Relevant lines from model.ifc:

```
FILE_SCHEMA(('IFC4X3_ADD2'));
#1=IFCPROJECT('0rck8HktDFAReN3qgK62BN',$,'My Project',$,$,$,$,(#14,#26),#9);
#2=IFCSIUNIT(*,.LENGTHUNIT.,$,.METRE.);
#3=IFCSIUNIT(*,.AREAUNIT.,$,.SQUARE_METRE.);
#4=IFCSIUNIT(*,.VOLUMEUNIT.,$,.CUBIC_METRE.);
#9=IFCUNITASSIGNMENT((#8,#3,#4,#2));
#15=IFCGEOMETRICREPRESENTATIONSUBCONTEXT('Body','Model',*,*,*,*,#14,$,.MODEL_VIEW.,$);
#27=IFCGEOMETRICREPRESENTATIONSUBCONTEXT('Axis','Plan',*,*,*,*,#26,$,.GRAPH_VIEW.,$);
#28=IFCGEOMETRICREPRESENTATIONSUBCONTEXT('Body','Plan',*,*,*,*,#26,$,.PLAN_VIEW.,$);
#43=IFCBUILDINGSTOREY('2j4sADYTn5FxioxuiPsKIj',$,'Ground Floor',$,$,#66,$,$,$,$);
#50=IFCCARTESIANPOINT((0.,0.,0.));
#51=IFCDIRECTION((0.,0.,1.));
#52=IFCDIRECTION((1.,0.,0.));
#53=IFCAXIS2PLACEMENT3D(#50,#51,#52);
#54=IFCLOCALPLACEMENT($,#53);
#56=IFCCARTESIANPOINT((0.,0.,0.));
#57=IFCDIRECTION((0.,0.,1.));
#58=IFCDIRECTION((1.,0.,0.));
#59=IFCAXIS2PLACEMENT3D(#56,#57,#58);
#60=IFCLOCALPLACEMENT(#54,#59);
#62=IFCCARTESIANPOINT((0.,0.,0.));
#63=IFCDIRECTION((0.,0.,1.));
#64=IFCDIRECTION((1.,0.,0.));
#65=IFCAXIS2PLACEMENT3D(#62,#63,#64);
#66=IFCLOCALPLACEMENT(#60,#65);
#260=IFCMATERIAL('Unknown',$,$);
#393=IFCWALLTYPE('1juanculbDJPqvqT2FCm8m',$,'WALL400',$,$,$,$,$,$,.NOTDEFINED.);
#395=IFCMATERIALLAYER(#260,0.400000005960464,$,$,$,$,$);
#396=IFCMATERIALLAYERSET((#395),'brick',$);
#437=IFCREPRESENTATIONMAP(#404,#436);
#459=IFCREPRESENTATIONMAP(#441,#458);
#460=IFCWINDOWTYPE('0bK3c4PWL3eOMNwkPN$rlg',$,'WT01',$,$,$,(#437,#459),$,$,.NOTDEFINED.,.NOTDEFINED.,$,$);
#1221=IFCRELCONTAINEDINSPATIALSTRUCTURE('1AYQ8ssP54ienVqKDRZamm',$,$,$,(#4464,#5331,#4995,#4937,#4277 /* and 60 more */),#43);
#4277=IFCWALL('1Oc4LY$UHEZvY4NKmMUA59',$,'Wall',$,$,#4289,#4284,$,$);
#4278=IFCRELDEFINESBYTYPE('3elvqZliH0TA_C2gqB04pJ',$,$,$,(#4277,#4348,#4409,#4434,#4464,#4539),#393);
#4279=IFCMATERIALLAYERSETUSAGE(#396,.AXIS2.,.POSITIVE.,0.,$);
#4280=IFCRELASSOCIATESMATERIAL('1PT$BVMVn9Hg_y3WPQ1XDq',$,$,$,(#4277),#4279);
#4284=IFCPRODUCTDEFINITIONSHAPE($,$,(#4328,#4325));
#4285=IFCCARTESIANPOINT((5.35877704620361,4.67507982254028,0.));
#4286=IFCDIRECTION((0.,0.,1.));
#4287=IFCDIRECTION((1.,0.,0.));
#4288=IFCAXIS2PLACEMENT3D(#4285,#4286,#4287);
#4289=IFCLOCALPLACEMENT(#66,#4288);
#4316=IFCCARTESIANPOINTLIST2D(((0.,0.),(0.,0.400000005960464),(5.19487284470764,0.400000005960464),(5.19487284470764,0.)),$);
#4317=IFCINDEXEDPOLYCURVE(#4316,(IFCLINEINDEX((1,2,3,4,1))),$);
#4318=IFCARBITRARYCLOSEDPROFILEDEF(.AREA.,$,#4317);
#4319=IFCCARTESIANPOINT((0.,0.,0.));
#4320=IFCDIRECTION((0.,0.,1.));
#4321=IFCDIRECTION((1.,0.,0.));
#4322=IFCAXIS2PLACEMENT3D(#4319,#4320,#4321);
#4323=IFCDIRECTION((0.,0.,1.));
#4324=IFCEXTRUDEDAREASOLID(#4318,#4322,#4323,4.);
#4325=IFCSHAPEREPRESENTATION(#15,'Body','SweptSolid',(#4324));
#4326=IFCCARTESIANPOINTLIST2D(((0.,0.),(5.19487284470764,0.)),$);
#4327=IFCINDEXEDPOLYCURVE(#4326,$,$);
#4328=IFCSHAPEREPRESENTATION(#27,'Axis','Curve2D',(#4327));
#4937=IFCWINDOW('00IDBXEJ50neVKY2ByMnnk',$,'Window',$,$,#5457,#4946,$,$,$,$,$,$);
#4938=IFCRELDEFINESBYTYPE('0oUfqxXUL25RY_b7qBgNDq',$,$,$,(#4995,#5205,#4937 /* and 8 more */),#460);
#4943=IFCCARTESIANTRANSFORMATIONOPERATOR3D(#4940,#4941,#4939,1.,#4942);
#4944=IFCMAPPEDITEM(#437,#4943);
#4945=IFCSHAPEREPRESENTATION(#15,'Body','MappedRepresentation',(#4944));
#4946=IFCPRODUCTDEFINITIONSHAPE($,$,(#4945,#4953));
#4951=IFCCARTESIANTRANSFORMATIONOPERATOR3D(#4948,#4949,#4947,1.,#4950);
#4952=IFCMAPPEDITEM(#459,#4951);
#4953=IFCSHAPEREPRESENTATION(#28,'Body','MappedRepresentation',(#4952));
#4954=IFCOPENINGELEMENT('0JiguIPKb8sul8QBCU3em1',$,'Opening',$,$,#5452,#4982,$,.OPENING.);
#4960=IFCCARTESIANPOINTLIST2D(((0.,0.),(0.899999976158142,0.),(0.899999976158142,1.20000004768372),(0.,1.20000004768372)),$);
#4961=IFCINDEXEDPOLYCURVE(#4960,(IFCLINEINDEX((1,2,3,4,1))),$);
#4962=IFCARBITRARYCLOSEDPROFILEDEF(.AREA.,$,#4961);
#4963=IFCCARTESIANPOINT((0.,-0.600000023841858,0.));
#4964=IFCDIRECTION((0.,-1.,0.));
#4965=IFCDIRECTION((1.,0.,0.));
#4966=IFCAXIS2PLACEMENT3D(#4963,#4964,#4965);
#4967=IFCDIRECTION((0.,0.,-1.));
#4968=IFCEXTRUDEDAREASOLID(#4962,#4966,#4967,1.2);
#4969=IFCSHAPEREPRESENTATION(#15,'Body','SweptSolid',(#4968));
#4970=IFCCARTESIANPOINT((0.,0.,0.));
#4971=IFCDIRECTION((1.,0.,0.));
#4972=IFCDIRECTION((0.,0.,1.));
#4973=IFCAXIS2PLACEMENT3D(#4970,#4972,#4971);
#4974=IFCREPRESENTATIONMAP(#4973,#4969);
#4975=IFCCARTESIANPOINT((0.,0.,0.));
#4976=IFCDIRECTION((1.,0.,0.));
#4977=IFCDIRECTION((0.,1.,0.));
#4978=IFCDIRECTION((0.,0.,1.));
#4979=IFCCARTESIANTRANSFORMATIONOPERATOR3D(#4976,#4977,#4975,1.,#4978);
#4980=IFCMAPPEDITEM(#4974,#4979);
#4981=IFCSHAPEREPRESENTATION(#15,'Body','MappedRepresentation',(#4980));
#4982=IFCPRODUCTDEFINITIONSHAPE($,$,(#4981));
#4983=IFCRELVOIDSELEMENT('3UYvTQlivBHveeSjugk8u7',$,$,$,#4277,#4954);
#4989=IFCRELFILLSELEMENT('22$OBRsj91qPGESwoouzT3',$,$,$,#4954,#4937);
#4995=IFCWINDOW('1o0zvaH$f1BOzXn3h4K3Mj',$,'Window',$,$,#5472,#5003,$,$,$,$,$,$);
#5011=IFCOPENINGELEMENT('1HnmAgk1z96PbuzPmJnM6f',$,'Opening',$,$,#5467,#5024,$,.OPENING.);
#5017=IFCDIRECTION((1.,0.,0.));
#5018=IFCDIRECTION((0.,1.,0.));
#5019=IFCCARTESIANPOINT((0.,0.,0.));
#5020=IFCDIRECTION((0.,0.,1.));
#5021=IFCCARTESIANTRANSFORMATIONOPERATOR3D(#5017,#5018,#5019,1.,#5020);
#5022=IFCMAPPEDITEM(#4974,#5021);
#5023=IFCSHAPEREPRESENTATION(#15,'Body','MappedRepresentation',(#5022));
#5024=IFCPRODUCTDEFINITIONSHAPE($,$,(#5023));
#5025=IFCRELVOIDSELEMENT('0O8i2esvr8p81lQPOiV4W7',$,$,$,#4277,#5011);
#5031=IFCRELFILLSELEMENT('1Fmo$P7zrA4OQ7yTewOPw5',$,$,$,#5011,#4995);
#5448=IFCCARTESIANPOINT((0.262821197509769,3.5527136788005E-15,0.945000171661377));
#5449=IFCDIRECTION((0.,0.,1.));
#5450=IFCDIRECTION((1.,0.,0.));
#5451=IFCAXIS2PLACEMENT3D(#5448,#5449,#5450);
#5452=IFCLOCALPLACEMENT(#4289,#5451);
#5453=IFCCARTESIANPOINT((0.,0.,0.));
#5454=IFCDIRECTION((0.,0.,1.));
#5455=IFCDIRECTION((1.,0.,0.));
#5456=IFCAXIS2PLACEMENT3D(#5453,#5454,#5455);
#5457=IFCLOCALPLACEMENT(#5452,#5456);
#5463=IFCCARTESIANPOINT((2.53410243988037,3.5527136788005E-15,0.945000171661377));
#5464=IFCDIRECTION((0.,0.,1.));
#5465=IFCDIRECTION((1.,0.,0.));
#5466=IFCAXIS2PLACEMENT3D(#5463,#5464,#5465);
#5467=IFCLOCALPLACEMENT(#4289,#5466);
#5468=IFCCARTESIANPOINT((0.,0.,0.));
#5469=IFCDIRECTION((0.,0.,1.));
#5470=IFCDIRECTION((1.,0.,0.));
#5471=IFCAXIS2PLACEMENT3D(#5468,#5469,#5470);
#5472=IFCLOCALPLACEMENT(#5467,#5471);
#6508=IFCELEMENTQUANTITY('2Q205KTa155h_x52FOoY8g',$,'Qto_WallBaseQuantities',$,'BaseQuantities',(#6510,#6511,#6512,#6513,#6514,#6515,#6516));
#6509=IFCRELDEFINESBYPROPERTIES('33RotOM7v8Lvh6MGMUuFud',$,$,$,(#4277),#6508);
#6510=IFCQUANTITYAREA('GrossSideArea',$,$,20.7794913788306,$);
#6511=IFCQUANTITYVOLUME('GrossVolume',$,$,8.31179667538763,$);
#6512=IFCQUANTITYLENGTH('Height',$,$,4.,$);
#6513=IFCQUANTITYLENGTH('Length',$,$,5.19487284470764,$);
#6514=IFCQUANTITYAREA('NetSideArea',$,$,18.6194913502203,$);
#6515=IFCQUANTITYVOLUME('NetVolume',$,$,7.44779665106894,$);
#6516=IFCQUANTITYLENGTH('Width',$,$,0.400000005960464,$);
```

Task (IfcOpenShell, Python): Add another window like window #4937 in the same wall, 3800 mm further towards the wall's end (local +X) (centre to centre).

```python
import ifcopenshell
import ifcopenshell.api.feature
import ifcopenshell.api.geometry
import ifcopenshell.api.pset
import ifcopenshell.api.root
import ifcopenshell.geom
import ifcopenshell.util.element
import ifcopenshell.util.placement
import ifcopenshell.util.shape
import ifcopenshell.util.unit

model = ifcopenshell.open("model.ifc")
unit_scale = ifcopenshell.util.unit.calculate_unit_scale(model)
area_scale = ifcopenshell.util.unit.calculate_unit_scale(model, "AREAUNIT")
volume_scale = ifcopenshell.util.unit.calculate_unit_scale(model, "VOLUMEUNIT")
settings = ifcopenshell.geom.settings()


def volume(element):
    """Net volume in cubic metres, openings subtracted."""
    shape = ifcopenshell.geom.create_shape(settings, element)
    return ifcopenshell.util.shape.get_volume(shape.geometry)


window = model.by_guid("00IDBXEJ50neVKY2ByMnnk")
opening = window.FillsVoids[0].RelatingOpeningElement
wall = opening.VoidsElements[0].RelatingBuildingElement
before = volume(wall)
shift = ifcopenshell.util.placement.get_local_placement(wall.ObjectPlacement)[:3, 0] * 3.8 / unit_scale

# copy_class copies the void relationship, type, container and properties, but no geometry.
new_opening = ifcopenshell.api.root.copy_class(model, product=opening)
new_opening.Representation = ifcopenshell.util.element.copy_deep(
    model, opening.Representation, exclude=["IfcGeometricRepresentationContext", "IfcRepresentationMap"]
)
new_window = ifcopenshell.api.root.copy_class(model, product=window)
new_window.Representation = ifcopenshell.util.element.copy_deep(
    model, window.Representation, exclude=["IfcGeometricRepresentationContext", "IfcRepresentationMap"]
)
ifcopenshell.api.feature.add_filling(model, opening=new_opening, element=new_window)

for old, new in ((opening, new_opening), (window, new_window)):
    matrix = ifcopenshell.util.placement.get_local_placement(old.ObjectPlacement)
    matrix[:3, 3] += shift
    ifcopenshell.api.geometry.edit_object_placement(model, product=new, matrix=matrix, is_si=False)

after = volume(wall)
thickness = 0.4  # wall thickness in metres

# Update the wall's stored quantities.
qto = model.by_id(ifcopenshell.util.element.get_pset(wall, "Qto_WallBaseQuantities", should_inherit=False)["id"])
ifcopenshell.api.pset.edit_qto(model, qto=qto, properties={
    "NetSideArea": after / thickness / area_scale,
    "NetVolume": after / volume_scale,
})

print(f"wall volume {before:.3f} -> {after:.3f} m3")

model.write("model_v2.ifc")
```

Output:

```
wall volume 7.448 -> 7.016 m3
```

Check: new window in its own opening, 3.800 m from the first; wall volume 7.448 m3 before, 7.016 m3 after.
